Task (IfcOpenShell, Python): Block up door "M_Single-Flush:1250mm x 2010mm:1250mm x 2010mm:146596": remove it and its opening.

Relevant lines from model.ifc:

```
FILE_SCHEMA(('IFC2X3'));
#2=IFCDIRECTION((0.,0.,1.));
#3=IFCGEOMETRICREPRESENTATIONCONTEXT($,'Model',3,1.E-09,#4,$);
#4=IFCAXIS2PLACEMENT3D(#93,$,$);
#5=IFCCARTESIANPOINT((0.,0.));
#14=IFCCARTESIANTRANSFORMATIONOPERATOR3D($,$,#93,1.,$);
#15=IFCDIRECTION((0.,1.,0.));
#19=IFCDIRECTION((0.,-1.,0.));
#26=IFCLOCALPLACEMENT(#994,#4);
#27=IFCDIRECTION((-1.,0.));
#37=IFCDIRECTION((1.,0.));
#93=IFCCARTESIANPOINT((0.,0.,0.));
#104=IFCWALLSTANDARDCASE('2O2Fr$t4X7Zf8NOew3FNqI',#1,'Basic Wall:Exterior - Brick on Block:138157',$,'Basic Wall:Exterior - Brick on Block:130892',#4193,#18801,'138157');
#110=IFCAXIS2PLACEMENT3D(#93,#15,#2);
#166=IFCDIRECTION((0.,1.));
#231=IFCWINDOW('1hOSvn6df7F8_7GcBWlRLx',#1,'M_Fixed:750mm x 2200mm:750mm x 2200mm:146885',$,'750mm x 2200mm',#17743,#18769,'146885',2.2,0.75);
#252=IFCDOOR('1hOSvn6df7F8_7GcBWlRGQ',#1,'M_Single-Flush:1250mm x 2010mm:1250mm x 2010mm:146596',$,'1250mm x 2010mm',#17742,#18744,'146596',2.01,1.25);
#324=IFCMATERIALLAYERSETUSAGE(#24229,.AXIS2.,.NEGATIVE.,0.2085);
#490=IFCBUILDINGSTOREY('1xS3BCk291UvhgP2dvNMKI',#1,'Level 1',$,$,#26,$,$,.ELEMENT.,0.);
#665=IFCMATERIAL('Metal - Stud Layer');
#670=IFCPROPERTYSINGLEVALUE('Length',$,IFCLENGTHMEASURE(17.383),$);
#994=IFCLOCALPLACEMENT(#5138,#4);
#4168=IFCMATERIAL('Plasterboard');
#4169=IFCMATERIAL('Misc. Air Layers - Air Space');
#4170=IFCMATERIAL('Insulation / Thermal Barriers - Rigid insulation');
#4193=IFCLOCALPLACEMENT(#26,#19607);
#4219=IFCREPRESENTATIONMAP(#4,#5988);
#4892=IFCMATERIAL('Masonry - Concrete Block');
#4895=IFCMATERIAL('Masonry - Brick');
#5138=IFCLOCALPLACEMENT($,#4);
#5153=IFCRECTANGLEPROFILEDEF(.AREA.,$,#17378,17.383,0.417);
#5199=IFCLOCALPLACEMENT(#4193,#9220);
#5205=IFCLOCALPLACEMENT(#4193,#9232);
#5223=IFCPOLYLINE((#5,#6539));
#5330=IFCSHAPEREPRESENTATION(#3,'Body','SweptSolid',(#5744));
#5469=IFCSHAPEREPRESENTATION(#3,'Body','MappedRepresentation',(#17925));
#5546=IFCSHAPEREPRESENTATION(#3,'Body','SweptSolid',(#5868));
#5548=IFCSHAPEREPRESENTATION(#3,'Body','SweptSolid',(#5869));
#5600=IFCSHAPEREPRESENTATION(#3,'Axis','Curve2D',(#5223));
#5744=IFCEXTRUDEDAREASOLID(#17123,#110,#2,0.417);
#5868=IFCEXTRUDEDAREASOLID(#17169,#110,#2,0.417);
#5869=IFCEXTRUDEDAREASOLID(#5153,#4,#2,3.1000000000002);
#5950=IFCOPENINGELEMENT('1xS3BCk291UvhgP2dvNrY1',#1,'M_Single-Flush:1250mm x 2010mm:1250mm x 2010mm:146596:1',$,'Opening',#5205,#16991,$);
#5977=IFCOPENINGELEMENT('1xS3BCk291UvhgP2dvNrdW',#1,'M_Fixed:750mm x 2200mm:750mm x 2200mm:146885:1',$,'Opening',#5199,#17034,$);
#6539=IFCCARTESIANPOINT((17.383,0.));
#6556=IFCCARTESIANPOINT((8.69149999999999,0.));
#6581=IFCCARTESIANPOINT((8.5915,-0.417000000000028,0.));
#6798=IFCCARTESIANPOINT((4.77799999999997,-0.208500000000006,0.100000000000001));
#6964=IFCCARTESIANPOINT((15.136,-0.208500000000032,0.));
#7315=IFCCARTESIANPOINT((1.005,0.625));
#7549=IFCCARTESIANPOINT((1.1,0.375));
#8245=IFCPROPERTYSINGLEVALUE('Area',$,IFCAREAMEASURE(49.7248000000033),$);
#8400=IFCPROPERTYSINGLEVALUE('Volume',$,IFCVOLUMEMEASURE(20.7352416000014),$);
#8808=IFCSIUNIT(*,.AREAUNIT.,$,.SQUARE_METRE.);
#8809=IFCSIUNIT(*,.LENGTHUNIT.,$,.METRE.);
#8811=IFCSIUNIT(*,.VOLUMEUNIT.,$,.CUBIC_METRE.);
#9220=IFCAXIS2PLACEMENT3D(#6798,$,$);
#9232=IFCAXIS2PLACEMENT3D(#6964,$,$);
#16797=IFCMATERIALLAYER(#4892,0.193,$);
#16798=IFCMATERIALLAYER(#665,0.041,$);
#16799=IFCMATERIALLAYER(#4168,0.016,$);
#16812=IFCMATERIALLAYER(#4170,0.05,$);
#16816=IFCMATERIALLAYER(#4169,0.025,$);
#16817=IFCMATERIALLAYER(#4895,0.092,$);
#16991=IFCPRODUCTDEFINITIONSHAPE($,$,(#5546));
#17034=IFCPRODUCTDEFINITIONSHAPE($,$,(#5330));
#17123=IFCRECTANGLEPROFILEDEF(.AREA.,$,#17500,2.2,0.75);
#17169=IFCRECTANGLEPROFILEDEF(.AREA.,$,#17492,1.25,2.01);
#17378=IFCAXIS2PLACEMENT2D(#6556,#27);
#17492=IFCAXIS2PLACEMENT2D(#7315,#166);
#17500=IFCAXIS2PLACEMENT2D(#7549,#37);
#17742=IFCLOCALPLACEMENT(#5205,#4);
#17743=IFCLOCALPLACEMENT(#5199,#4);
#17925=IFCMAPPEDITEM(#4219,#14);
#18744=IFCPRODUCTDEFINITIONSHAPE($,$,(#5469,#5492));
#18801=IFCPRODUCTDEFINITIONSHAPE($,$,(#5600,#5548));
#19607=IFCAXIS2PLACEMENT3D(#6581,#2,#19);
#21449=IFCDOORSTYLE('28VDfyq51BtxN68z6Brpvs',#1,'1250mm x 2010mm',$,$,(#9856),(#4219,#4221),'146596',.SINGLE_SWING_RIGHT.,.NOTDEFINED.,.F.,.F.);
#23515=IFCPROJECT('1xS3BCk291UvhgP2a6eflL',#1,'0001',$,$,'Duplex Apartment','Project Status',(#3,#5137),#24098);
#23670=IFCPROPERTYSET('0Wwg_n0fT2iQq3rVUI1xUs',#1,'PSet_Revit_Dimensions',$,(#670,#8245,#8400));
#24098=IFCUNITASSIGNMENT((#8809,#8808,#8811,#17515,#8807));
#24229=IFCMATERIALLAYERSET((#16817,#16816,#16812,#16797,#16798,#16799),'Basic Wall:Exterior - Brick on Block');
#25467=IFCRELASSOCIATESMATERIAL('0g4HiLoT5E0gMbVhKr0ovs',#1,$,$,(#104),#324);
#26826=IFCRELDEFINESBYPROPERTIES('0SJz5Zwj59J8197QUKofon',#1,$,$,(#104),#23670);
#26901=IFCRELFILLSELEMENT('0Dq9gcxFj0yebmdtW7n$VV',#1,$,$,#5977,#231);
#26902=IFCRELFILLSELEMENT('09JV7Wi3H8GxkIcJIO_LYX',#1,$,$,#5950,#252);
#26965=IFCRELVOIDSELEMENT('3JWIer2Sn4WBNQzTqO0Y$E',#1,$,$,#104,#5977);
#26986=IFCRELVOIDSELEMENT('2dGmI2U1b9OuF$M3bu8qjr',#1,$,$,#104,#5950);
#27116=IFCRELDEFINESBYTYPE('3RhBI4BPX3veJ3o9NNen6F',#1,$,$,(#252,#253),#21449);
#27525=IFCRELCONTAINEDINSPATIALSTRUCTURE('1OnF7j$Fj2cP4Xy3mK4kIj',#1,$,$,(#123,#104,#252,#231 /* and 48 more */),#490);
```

```python
import ifcopenshell
import ifcopenshell.api.feature
import ifcopenshell.api.pset
import ifcopenshell.api.root
import ifcopenshell.geom
import ifcopenshell.util.element
import ifcopenshell.util.shape
import ifcopenshell.util.unit

model = ifcopenshell.open("model.ifc")
area_scale = ifcopenshell.util.unit.calculate_unit_scale(model, "AREAUNIT")
volume_scale = ifcopenshell.util.unit.calculate_unit_scale(model, "VOLUMEUNIT")
settings = ifcopenshell.geom.settings()


def volume(element):
    """Net volume in cubic metres, openings subtracted."""
    shape = ifcopenshell.geom.create_shape(settings, element)
    return ifcopenshell.util.shape.get_volume(shape.geometry)


door = model.by_guid("1hOSvn6df7F8_7GcBWlRGQ")
opening = door.FillsVoids[0].RelatingOpeningElement
wall = opening.VoidsElements[0].RelatingBuildingElement
before = volume(wall)

ifcopenshell.api.root.remove_product(model, product=door)
ifcopenshell.api.feature.remove_feature(model, feature=opening)

after = volume(wall)
thickness = 0.417  # wall thickness in metres

# Update the wall's stored quantities.
pset = model.by_id(ifcopenshell.util.element.get_pset(wall, "PSet_Revit_Dimensions", should_inherit=False)["id"])
ifcopenshell.api.pset.edit_pset(model, pset=pset, properties={
    "Area": model.create_entity("IfcAreaMeasure", after / thickness / area_scale),
    "Volume": model.create_entity("IfcVolumeMeasure", after / volume_scale),
})

print(f"wall volume {before:.3f} -> {after:.3f} m3")

model.write("model_v2.ifc")
```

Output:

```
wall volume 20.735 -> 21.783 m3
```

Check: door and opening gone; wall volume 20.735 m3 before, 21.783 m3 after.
